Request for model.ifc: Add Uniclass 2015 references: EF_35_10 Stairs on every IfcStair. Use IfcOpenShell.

First a look at what the model holds.

```python
import ifcopenshell

model = ifcopenshell.open("model.ifc")
print(model.schema)
print("classifications:", [c.Name for c in model.by_type("IfcClassification")])
for ifc_class in ("IfcDoor", "IfcRoof", "IfcStair", "IfcWall", "IfcWindow"):
    print(ifc_class, len(model.by_type(ifc_class)))
```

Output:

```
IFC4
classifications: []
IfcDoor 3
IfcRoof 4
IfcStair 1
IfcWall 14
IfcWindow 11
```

```python
import ifcopenshell
import ifcopenshell.api.classification

model = ifcopenshell.open("model.ifc")

system = ifcopenshell.api.classification.add_classification(model, classification="Uniclass 2015")

codes = {
    "IfcStair": ("EF_35_10", "Stairs"),
}
for ifc_class, (code, name) in codes.items():
    products = model.by_type(ifc_class)
    ifcopenshell.api.classification.add_reference(
        model, products=products, classification=system, identification=code, name=name
    )
    print(code, len(products))

model.write("model_edited.ifc")
```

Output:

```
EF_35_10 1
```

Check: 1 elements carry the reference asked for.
